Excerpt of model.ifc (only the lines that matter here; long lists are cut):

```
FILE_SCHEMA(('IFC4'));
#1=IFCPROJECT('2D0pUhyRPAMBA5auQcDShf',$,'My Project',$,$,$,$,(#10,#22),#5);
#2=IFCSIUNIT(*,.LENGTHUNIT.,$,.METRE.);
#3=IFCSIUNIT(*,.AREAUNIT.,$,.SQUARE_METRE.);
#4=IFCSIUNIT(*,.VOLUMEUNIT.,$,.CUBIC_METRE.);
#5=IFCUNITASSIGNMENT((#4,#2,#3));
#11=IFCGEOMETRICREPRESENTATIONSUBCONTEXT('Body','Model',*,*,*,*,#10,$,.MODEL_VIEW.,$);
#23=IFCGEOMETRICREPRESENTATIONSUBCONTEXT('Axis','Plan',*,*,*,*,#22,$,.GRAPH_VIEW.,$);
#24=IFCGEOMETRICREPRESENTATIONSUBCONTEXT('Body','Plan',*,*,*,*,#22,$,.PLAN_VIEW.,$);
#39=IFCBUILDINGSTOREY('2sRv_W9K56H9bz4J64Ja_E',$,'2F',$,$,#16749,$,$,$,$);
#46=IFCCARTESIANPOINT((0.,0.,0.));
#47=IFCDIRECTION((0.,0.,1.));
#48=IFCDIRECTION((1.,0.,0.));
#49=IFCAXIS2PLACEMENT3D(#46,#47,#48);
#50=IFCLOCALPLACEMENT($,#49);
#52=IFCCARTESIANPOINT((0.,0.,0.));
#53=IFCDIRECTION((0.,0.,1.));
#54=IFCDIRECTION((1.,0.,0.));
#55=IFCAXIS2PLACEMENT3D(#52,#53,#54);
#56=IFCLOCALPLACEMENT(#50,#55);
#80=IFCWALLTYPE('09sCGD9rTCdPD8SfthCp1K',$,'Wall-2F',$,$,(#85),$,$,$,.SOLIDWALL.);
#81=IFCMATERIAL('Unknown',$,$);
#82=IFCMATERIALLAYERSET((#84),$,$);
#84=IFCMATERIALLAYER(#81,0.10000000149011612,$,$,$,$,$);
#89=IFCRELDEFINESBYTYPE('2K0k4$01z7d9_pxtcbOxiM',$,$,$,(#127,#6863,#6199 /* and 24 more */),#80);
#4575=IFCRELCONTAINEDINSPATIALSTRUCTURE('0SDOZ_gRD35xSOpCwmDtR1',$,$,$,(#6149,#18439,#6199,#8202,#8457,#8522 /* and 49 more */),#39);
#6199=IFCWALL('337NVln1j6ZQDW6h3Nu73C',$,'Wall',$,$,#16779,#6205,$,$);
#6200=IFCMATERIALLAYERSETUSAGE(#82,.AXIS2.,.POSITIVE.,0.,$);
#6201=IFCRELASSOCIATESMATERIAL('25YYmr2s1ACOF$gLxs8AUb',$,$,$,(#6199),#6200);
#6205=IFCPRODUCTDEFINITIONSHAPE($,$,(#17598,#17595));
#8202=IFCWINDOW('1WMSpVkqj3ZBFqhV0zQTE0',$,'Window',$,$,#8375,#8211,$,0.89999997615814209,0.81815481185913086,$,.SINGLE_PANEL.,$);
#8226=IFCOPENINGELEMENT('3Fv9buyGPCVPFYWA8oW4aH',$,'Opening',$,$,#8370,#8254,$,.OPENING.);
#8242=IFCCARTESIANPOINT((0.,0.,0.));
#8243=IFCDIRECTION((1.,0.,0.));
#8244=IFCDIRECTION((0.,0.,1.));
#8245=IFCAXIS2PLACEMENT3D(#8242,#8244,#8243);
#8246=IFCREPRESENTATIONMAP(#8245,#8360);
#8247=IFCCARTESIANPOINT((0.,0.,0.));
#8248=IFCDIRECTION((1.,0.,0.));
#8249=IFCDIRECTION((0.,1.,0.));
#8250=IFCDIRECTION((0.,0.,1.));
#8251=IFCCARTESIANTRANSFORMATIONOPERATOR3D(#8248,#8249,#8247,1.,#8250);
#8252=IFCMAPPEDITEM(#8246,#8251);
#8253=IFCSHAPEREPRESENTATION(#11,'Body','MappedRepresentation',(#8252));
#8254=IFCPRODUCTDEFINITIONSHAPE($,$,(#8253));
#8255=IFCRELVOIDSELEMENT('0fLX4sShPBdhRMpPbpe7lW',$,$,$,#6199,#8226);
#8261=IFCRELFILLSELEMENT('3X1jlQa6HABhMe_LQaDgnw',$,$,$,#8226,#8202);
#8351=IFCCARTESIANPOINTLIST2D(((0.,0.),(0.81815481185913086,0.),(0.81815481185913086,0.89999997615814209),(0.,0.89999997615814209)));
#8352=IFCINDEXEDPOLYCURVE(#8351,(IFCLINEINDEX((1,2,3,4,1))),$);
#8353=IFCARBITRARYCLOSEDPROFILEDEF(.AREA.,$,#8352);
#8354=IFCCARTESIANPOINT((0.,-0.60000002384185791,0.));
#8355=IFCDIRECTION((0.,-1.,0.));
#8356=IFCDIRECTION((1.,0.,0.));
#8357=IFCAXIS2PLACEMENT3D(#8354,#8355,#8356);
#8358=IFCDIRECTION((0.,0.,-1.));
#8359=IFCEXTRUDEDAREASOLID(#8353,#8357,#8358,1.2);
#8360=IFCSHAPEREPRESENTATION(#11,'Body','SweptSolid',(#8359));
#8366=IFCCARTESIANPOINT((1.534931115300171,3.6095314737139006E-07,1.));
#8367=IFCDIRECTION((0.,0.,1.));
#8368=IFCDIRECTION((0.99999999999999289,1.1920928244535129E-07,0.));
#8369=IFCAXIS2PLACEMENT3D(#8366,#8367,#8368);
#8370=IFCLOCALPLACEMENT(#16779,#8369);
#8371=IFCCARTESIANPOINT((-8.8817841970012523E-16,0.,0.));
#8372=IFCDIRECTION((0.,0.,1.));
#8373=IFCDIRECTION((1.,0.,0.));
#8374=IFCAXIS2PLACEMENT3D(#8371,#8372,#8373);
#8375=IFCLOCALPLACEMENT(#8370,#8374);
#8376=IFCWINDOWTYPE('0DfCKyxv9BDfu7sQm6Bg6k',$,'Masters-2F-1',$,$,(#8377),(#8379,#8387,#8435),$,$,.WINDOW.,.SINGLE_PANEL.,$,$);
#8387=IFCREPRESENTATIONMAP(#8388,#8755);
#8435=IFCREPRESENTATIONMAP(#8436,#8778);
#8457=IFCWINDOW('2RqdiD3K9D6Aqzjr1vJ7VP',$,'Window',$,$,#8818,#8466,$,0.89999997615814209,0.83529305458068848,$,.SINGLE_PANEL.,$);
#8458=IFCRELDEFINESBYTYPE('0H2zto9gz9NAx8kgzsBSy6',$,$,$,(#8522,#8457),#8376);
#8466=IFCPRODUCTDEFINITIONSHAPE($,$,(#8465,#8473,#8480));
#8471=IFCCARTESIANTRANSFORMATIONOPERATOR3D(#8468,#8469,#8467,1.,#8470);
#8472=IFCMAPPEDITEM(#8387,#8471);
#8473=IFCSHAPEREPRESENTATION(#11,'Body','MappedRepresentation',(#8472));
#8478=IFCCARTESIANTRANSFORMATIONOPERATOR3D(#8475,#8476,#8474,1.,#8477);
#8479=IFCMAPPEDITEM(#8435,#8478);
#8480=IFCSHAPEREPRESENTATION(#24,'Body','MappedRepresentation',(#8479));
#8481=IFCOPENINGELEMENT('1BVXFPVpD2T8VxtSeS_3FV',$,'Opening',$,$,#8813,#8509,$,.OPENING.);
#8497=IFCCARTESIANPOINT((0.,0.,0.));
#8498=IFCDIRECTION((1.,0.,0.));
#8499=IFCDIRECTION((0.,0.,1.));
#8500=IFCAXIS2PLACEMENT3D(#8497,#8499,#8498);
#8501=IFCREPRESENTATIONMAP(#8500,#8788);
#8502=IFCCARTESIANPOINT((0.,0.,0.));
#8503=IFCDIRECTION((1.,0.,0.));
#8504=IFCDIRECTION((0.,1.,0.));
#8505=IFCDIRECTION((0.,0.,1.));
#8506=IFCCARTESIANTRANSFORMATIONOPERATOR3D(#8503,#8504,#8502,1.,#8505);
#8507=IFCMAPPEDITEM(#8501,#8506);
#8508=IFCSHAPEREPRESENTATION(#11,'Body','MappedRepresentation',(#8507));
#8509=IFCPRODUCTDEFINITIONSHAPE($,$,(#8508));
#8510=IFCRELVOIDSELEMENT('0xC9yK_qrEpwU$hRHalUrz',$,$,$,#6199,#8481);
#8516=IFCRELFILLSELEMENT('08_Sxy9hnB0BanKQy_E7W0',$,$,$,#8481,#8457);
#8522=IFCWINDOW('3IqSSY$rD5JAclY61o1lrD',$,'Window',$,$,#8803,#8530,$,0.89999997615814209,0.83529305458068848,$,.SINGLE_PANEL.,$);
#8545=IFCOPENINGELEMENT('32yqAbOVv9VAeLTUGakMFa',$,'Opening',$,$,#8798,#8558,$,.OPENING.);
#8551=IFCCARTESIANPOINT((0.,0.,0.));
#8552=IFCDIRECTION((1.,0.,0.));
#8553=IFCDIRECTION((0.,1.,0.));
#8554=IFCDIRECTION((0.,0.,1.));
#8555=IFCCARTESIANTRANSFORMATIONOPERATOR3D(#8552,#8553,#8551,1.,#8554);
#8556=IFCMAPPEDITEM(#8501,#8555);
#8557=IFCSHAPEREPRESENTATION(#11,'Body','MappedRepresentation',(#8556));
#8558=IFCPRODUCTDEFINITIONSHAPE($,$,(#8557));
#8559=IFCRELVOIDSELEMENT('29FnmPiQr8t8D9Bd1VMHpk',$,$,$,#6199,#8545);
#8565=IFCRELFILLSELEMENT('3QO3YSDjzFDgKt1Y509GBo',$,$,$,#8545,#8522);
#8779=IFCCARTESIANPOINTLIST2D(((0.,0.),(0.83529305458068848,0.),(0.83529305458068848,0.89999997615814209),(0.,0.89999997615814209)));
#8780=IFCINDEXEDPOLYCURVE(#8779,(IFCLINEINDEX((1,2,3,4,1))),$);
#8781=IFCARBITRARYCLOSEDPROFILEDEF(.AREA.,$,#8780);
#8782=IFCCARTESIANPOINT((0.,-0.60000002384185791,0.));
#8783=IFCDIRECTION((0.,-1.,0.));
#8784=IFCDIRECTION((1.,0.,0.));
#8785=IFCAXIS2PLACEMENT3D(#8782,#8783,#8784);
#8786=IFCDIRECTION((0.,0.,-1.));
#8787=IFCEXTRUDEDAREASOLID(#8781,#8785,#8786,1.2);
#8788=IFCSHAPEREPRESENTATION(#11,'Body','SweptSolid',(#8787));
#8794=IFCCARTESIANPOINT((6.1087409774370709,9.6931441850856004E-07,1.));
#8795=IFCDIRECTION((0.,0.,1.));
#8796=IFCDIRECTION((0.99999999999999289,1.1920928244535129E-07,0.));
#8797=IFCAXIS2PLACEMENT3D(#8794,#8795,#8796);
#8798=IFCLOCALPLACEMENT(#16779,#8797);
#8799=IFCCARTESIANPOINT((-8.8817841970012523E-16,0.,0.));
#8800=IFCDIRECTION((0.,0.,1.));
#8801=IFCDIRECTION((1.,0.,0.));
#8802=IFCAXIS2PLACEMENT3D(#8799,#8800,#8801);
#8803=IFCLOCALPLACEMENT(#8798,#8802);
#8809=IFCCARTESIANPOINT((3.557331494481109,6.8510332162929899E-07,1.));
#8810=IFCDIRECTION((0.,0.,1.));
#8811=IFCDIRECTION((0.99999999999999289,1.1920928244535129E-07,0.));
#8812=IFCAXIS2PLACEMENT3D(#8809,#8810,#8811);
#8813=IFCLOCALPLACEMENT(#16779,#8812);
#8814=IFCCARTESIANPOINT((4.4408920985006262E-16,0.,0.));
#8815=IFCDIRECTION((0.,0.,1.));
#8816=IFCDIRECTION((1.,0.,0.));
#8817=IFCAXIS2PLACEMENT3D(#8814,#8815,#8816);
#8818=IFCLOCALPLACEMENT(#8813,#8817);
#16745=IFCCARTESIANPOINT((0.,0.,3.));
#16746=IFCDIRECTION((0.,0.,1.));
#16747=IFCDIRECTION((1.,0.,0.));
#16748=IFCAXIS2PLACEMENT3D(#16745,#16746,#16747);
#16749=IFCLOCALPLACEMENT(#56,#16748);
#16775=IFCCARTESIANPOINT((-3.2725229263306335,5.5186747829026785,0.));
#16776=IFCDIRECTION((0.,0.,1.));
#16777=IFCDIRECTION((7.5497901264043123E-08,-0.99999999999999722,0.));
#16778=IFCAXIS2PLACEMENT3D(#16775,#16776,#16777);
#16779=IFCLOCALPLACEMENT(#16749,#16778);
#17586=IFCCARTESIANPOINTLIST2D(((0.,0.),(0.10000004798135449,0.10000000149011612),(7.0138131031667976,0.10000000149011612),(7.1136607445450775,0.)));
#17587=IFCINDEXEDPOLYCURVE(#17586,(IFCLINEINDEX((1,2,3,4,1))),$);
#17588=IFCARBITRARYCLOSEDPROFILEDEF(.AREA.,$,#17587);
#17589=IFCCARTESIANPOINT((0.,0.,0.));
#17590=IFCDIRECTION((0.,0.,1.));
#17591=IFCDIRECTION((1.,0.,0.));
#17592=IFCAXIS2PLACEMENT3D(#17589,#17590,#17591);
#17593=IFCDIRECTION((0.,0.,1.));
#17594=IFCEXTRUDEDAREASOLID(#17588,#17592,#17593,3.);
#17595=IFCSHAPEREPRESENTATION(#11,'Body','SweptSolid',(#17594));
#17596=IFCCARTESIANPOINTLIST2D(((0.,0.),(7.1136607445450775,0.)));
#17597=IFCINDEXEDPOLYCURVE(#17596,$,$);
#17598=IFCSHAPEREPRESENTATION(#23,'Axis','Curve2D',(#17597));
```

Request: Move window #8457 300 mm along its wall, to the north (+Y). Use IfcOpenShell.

```python
import ifcopenshell
import ifcopenshell.api.geometry
import ifcopenshell.util.placement
import ifcopenshell.util.unit

model = ifcopenshell.open("model.ifc")
unit_scale = ifcopenshell.util.unit.calculate_unit_scale(model)

window = model.by_guid("2RqdiD3K9D6Aqzjr1vJ7VP")
opening = window.FillsVoids[0].RelatingOpeningElement
wall = opening.VoidsElements[0].RelatingBuildingElement

wall_matrix = ifcopenshell.util.placement.get_local_placement(wall.ObjectPlacement)
shift = wall_matrix[:3, 0] * -0.3 / unit_scale
before = ifcopenshell.util.placement.get_local_placement(window.ObjectPlacement)[:3, 3].copy()

# The window is placed relative to its opening, so it follows when the opening moves.
matrix = ifcopenshell.util.placement.get_local_placement(opening.ObjectPlacement)
matrix[:3, 3] += shift
ifcopenshell.api.geometry.edit_object_placement(
    model, product=opening, matrix=matrix, is_si=False, should_transform_children=True
)

after = ifcopenshell.util.placement.get_local_placement(window.ObjectPlacement)[:3, 3]
print("window moved by", (after - before).round(3) + 0.0)

model.write("model-out.ifc")
```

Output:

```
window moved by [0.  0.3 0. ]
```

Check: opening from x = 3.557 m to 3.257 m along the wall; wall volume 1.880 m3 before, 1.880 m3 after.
